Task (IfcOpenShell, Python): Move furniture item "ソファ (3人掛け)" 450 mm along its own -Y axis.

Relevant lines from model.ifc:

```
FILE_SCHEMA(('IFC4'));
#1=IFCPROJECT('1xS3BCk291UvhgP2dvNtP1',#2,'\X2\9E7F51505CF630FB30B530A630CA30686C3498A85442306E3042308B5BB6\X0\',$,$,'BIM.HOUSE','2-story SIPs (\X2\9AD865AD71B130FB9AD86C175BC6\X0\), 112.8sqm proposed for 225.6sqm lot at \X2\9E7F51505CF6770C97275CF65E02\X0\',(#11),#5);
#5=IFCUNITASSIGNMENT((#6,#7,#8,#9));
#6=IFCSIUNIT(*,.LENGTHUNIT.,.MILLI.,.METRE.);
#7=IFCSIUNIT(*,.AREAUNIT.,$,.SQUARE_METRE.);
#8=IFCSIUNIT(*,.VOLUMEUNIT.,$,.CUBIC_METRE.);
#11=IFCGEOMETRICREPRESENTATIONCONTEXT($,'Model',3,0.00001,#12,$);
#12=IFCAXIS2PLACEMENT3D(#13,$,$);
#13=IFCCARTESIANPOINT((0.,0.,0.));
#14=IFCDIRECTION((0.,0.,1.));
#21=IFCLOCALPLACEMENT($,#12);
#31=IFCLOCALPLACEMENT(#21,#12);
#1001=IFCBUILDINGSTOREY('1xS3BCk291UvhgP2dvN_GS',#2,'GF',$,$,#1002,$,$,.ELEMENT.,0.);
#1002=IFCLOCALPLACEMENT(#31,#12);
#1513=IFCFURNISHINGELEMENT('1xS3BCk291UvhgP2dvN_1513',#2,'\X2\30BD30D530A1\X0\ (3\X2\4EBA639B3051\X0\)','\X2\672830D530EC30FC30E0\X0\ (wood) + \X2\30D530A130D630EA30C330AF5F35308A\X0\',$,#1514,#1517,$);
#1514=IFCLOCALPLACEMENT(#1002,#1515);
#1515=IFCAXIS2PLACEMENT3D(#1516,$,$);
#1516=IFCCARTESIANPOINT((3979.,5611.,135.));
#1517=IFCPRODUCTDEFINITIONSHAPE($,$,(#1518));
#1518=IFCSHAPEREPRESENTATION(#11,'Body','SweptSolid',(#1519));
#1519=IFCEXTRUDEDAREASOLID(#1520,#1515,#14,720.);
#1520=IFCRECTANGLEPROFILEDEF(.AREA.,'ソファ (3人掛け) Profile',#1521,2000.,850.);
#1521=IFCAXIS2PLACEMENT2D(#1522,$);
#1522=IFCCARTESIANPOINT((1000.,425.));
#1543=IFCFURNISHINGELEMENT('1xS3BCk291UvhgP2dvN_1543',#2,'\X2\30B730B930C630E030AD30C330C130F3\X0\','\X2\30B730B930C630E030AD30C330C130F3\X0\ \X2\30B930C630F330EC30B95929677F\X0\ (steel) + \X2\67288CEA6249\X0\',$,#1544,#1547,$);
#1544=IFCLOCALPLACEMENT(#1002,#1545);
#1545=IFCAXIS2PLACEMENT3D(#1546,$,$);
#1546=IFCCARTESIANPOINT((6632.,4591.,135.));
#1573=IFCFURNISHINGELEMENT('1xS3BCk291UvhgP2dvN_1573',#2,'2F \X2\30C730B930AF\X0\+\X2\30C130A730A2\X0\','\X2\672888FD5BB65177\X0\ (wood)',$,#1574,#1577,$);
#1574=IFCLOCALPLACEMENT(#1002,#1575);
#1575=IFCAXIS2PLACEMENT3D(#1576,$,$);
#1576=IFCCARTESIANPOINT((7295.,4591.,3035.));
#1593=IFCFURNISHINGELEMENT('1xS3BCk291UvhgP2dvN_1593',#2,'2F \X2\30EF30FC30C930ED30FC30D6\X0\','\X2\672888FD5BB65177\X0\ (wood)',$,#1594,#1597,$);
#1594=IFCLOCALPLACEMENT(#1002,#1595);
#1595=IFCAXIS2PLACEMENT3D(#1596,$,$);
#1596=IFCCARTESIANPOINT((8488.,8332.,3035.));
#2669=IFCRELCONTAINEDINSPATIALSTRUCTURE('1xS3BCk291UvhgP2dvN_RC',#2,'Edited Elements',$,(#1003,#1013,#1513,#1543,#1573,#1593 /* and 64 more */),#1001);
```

```python
import ifcopenshell
import ifcopenshell.api.geometry
import ifcopenshell.util.placement
import ifcopenshell.util.unit

model = ifcopenshell.open("model.ifc")
unit_scale = ifcopenshell.util.unit.calculate_unit_scale(model)

item = model.by_guid("1xS3BCk291UvhgP2dvN_1513")
matrix = ifcopenshell.util.placement.get_local_placement(item.ObjectPlacement)
matrix[:3, 3] -= matrix[:3, 1] * 0.45 / unit_scale
ifcopenshell.api.geometry.edit_object_placement(model, product=item, matrix=matrix, is_si=False)

print(ifcopenshell.util.placement.get_local_placement(item.ObjectPlacement).round(3) + 0.0)

model.write("model_edited.ifc")
```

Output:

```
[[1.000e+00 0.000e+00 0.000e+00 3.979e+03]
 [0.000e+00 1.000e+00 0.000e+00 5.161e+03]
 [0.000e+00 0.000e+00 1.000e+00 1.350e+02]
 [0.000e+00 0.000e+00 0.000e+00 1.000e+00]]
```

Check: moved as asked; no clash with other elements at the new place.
